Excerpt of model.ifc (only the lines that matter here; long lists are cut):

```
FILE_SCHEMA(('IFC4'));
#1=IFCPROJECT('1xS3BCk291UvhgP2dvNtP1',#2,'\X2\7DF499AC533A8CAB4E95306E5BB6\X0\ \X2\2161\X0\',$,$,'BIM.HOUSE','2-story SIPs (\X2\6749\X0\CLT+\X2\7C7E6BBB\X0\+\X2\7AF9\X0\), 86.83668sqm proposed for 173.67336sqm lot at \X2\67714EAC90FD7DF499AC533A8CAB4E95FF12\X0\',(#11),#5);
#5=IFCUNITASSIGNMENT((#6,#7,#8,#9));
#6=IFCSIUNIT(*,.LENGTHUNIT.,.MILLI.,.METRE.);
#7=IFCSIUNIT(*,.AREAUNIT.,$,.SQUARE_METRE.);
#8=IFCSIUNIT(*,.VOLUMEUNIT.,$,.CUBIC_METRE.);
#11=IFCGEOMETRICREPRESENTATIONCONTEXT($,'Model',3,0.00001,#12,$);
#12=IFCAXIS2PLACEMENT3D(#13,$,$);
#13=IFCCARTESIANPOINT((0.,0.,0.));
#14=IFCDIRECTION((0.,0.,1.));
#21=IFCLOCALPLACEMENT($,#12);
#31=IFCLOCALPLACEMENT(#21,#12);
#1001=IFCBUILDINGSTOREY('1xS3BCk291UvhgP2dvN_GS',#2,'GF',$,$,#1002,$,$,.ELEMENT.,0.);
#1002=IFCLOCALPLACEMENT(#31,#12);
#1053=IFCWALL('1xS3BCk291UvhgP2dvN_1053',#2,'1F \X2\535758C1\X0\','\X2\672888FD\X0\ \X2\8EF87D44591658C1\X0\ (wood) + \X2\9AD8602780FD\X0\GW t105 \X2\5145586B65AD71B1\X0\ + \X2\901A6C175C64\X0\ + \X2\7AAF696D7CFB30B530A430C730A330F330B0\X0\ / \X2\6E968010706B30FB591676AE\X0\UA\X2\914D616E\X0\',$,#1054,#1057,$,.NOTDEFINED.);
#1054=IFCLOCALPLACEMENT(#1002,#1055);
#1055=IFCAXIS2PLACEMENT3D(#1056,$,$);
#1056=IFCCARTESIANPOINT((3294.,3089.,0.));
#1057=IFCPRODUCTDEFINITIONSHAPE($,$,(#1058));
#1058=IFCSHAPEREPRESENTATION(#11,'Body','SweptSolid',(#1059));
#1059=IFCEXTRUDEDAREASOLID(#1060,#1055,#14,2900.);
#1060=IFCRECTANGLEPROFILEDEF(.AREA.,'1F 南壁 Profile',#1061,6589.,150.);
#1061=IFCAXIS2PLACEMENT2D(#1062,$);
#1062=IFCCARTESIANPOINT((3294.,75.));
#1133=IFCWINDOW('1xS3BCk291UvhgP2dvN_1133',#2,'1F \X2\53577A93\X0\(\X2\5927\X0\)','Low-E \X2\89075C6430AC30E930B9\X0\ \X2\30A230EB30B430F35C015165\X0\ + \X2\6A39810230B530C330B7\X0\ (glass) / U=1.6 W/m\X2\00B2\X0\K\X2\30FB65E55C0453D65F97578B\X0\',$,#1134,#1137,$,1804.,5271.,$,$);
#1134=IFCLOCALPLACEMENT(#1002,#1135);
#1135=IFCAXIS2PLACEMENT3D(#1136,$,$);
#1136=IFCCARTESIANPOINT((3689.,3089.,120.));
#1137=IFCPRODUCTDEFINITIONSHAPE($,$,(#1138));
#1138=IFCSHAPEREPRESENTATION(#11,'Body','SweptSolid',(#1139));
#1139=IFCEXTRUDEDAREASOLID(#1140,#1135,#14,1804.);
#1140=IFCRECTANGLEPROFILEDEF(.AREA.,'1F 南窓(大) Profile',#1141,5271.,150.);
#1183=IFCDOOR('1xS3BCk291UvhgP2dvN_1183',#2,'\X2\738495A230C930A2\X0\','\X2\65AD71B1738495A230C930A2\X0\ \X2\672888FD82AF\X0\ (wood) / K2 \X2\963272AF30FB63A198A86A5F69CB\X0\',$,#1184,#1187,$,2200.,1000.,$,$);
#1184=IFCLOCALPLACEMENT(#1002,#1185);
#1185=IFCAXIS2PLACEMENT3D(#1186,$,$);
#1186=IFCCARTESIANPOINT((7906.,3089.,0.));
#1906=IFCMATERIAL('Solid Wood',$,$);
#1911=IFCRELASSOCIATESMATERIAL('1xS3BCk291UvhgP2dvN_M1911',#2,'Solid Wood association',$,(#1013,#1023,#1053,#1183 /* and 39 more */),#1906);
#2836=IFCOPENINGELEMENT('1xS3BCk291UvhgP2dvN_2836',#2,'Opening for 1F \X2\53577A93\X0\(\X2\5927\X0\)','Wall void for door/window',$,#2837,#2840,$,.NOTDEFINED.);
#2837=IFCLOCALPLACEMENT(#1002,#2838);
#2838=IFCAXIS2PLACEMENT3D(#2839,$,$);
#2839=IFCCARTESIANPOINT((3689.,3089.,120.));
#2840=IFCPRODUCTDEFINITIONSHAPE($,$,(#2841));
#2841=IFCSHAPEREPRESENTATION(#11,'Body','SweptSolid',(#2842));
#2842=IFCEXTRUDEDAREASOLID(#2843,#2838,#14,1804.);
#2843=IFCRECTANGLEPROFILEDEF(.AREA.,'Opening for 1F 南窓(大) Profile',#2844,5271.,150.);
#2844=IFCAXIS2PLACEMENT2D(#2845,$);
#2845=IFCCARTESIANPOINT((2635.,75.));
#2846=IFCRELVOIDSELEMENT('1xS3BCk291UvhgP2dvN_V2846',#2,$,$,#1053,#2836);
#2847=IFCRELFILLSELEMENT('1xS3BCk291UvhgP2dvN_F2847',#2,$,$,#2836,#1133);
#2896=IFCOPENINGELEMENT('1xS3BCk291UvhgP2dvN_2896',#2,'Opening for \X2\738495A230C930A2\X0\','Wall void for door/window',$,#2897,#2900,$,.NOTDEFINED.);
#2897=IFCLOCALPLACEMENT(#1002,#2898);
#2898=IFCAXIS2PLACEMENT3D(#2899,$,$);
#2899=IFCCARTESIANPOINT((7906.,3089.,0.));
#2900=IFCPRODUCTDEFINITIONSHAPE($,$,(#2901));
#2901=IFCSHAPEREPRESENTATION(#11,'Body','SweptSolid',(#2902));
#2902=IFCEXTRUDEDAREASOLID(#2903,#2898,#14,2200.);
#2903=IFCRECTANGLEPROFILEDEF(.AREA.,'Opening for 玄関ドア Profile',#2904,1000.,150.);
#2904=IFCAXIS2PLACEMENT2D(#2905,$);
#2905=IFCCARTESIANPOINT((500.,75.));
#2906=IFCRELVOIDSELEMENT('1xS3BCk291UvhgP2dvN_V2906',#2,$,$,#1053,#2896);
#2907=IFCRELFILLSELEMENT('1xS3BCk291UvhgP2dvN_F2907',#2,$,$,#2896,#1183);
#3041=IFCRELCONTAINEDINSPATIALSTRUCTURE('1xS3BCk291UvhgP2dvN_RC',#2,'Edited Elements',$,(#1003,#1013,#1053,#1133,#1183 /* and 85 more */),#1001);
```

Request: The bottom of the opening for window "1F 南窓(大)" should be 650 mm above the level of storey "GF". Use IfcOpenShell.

```python
import numpy as np
import ifcopenshell
import ifcopenshell.api.geometry
import ifcopenshell.geom
import ifcopenshell.util.element
import ifcopenshell.util.placement
import ifcopenshell.util.shape
import ifcopenshell.util.unit

model = ifcopenshell.open("model.ifc")
unit_scale = ifcopenshell.util.unit.calculate_unit_scale(model)

window = model.by_guid("1xS3BCk291UvhgP2dvN_1133")
opening = window.FillsVoids[0].RelatingOpeningElement
storey = ifcopenshell.util.element.get_container(window, ifc_class="IfcBuildingStorey")
level = ifcopenshell.util.placement.get_local_placement(storey.ObjectPlacement)[2, 3]

# The opening's origin need not be at the sill, so measure its lowest point.
shape = ifcopenshell.geom.create_shape(ifcopenshell.geom.settings(), opening)
bottom = ifcopenshell.util.shape.get_shape_bottom_elevation(shape, shape.geometry) / unit_scale
dz = level + 650.0 - bottom

shift = np.array([0.0, 0.0, dz])
# The window is not placed relative to its opening, so move both.
for product in (opening, window):
    matrix = ifcopenshell.util.placement.get_local_placement(product.ObjectPlacement)
    matrix[:3, 3] += shift
    ifcopenshell.api.geometry.edit_object_placement(model, product=product, matrix=matrix, is_si=False)

print(f"moved by {dz * unit_scale:+.3f} m")

model.write("model_rev.ifc")
```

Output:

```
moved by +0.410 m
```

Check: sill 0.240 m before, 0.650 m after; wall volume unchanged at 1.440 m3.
